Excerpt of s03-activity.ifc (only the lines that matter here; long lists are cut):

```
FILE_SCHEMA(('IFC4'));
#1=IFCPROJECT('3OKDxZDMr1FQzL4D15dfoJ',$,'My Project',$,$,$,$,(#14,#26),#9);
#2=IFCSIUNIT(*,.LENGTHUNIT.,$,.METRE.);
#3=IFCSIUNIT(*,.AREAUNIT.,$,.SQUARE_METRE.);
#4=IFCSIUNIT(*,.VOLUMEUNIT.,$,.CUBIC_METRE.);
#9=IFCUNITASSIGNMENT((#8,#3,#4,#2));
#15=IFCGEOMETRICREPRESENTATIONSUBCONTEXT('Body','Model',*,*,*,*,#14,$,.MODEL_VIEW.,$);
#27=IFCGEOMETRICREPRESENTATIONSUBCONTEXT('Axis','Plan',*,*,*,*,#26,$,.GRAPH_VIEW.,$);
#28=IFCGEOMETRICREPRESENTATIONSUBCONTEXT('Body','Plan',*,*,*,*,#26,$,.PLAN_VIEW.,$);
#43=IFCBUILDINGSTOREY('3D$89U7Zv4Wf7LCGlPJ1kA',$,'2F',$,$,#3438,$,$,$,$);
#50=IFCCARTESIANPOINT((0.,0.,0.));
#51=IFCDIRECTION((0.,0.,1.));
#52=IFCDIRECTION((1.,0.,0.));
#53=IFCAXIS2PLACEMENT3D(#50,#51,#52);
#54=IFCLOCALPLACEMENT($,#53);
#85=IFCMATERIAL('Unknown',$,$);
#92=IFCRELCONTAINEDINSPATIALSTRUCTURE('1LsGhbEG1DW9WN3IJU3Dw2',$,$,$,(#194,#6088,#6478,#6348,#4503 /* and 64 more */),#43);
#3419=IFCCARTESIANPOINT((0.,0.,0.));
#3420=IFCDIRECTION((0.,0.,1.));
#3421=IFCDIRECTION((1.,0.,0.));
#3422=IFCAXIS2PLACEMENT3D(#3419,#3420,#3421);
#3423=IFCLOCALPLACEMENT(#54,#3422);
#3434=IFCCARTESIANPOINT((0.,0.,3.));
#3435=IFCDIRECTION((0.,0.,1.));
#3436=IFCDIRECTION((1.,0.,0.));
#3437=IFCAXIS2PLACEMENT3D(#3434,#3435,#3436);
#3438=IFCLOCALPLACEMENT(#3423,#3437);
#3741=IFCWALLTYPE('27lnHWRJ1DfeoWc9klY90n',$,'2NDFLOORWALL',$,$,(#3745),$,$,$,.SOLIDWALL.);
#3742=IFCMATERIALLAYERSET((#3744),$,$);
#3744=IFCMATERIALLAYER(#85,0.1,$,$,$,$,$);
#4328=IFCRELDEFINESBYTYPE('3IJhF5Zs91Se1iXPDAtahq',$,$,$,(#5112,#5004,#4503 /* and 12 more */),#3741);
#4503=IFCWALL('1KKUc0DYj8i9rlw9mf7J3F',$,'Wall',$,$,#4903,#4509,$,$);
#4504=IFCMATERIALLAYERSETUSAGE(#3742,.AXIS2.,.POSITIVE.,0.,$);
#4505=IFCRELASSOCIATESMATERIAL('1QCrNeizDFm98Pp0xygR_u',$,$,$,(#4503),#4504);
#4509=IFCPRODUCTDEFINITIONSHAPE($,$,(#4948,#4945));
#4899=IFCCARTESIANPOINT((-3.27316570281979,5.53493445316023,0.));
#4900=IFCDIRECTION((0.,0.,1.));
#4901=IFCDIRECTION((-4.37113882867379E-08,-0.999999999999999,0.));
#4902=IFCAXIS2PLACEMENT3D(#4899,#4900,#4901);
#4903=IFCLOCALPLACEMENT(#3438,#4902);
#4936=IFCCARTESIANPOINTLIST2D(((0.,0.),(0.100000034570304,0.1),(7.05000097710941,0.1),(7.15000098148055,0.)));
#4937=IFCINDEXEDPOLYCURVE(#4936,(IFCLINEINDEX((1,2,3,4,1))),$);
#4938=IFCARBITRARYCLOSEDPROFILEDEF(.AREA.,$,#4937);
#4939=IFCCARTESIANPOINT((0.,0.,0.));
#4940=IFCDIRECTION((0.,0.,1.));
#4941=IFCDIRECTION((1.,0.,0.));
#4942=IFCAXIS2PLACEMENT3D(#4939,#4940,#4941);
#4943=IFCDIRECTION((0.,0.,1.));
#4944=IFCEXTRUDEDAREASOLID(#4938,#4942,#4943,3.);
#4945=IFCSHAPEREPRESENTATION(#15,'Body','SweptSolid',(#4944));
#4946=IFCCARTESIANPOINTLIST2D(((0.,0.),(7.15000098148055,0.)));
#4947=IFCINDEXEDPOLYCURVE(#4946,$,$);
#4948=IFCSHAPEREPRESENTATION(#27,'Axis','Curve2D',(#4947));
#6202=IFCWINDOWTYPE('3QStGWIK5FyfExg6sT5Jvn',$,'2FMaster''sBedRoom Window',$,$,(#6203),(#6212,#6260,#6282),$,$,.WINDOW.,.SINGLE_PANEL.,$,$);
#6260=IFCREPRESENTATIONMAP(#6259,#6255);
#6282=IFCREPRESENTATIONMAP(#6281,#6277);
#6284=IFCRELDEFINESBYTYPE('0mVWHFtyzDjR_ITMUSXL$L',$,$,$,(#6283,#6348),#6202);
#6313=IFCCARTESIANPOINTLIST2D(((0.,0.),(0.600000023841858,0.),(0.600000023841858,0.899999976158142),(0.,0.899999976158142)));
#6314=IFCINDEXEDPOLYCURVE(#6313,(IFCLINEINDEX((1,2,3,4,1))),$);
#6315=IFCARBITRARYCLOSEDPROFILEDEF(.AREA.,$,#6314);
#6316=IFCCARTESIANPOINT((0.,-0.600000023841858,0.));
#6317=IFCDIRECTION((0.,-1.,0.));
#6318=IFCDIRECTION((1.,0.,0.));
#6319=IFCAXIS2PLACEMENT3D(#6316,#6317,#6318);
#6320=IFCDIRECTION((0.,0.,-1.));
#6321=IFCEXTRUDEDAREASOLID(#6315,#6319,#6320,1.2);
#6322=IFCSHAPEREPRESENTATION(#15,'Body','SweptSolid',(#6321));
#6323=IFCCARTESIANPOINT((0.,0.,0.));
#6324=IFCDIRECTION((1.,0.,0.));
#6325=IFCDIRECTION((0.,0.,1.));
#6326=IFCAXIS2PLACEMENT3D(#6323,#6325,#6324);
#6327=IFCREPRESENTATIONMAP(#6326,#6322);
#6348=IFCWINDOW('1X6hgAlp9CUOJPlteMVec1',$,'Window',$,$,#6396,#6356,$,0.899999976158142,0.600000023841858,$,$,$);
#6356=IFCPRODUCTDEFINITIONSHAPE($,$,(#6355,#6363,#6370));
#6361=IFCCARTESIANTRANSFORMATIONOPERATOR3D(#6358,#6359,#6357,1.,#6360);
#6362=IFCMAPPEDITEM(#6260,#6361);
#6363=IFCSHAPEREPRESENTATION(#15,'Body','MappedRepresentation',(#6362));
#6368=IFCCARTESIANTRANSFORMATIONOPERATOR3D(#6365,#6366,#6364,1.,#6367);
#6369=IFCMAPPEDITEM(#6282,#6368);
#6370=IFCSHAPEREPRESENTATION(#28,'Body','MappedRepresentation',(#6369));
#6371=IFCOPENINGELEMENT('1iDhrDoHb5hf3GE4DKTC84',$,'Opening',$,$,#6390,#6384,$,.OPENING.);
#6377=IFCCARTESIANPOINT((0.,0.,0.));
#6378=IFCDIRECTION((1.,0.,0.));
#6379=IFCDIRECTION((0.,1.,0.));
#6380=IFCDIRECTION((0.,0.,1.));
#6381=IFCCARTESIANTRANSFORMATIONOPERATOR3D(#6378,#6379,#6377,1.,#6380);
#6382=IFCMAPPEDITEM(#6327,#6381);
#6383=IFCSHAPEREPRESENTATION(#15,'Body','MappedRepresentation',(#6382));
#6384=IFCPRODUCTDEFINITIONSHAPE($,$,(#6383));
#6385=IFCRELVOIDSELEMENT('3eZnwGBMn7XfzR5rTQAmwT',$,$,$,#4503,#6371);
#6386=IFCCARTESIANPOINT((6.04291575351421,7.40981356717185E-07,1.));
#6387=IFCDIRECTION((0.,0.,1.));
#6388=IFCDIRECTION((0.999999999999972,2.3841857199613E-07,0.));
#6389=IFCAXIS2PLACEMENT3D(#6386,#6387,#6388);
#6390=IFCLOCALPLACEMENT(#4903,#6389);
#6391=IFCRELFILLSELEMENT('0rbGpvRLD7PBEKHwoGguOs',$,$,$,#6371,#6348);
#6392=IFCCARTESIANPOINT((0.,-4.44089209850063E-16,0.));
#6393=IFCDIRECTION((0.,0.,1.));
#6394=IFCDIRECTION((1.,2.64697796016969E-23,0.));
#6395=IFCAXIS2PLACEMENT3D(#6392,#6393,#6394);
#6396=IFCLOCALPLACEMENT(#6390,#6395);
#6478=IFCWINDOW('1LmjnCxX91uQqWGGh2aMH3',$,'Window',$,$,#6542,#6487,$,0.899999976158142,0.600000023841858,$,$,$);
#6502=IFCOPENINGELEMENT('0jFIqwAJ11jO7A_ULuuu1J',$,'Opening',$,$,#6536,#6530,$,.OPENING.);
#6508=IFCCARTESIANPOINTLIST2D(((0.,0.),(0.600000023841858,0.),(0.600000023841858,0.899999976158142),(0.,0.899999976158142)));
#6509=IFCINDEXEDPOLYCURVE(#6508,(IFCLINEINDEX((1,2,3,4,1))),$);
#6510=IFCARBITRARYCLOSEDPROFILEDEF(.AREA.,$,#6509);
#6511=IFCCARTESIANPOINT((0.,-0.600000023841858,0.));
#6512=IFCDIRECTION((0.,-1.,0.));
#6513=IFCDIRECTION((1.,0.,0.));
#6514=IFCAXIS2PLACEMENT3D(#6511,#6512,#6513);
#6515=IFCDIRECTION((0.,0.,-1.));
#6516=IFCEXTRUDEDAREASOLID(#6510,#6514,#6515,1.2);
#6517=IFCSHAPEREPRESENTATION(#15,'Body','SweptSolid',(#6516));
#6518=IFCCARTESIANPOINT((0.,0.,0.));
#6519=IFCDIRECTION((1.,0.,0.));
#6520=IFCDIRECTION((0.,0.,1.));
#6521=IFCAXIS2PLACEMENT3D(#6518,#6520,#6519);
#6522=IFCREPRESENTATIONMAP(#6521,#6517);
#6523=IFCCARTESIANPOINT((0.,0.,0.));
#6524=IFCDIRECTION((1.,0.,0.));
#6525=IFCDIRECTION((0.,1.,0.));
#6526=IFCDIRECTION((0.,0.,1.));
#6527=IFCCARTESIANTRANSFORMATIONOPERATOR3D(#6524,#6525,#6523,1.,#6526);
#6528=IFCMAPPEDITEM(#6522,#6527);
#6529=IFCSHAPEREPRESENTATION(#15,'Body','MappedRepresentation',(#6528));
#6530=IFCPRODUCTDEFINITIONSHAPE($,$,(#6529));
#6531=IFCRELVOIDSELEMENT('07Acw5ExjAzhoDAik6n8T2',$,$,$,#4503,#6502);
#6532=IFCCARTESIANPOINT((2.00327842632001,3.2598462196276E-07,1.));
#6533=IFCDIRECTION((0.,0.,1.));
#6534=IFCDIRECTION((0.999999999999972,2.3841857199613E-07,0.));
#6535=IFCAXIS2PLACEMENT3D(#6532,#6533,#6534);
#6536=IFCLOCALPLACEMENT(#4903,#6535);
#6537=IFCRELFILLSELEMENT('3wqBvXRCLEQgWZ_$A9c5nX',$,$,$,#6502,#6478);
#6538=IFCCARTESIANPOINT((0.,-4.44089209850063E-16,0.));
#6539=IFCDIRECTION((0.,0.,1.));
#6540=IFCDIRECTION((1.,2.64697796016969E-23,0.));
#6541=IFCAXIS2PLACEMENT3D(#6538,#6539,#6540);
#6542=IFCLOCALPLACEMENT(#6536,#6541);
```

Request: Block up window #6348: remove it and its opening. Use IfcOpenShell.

```python
import ifcopenshell
import ifcopenshell.api.feature
import ifcopenshell.api.root
import ifcopenshell.geom
import ifcopenshell.util.shape

model = ifcopenshell.open("s03-activity.ifc")
settings = ifcopenshell.geom.settings()


def volume(element):
    """Net volume in cubic metres, openings subtracted."""
    shape = ifcopenshell.geom.create_shape(settings, element)
    return ifcopenshell.util.shape.get_volume(shape.geometry)


window = model.by_guid("1X6hgAlp9CUOJPlteMVec1")
opening = window.FillsVoids[0].RelatingOpeningElement
wall = opening.VoidsElements[0].RelatingBuildingElement
before = volume(wall)

ifcopenshell.api.root.remove_product(model, product=window)
ifcopenshell.api.feature.remove_feature(model, feature=opening)

after = volume(wall)

print(f"wall volume {before:.3f} -> {after:.3f} m3")

model.write("s03-activity_v2.ifc")
```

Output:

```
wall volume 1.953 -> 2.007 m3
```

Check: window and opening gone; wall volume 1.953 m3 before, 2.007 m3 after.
